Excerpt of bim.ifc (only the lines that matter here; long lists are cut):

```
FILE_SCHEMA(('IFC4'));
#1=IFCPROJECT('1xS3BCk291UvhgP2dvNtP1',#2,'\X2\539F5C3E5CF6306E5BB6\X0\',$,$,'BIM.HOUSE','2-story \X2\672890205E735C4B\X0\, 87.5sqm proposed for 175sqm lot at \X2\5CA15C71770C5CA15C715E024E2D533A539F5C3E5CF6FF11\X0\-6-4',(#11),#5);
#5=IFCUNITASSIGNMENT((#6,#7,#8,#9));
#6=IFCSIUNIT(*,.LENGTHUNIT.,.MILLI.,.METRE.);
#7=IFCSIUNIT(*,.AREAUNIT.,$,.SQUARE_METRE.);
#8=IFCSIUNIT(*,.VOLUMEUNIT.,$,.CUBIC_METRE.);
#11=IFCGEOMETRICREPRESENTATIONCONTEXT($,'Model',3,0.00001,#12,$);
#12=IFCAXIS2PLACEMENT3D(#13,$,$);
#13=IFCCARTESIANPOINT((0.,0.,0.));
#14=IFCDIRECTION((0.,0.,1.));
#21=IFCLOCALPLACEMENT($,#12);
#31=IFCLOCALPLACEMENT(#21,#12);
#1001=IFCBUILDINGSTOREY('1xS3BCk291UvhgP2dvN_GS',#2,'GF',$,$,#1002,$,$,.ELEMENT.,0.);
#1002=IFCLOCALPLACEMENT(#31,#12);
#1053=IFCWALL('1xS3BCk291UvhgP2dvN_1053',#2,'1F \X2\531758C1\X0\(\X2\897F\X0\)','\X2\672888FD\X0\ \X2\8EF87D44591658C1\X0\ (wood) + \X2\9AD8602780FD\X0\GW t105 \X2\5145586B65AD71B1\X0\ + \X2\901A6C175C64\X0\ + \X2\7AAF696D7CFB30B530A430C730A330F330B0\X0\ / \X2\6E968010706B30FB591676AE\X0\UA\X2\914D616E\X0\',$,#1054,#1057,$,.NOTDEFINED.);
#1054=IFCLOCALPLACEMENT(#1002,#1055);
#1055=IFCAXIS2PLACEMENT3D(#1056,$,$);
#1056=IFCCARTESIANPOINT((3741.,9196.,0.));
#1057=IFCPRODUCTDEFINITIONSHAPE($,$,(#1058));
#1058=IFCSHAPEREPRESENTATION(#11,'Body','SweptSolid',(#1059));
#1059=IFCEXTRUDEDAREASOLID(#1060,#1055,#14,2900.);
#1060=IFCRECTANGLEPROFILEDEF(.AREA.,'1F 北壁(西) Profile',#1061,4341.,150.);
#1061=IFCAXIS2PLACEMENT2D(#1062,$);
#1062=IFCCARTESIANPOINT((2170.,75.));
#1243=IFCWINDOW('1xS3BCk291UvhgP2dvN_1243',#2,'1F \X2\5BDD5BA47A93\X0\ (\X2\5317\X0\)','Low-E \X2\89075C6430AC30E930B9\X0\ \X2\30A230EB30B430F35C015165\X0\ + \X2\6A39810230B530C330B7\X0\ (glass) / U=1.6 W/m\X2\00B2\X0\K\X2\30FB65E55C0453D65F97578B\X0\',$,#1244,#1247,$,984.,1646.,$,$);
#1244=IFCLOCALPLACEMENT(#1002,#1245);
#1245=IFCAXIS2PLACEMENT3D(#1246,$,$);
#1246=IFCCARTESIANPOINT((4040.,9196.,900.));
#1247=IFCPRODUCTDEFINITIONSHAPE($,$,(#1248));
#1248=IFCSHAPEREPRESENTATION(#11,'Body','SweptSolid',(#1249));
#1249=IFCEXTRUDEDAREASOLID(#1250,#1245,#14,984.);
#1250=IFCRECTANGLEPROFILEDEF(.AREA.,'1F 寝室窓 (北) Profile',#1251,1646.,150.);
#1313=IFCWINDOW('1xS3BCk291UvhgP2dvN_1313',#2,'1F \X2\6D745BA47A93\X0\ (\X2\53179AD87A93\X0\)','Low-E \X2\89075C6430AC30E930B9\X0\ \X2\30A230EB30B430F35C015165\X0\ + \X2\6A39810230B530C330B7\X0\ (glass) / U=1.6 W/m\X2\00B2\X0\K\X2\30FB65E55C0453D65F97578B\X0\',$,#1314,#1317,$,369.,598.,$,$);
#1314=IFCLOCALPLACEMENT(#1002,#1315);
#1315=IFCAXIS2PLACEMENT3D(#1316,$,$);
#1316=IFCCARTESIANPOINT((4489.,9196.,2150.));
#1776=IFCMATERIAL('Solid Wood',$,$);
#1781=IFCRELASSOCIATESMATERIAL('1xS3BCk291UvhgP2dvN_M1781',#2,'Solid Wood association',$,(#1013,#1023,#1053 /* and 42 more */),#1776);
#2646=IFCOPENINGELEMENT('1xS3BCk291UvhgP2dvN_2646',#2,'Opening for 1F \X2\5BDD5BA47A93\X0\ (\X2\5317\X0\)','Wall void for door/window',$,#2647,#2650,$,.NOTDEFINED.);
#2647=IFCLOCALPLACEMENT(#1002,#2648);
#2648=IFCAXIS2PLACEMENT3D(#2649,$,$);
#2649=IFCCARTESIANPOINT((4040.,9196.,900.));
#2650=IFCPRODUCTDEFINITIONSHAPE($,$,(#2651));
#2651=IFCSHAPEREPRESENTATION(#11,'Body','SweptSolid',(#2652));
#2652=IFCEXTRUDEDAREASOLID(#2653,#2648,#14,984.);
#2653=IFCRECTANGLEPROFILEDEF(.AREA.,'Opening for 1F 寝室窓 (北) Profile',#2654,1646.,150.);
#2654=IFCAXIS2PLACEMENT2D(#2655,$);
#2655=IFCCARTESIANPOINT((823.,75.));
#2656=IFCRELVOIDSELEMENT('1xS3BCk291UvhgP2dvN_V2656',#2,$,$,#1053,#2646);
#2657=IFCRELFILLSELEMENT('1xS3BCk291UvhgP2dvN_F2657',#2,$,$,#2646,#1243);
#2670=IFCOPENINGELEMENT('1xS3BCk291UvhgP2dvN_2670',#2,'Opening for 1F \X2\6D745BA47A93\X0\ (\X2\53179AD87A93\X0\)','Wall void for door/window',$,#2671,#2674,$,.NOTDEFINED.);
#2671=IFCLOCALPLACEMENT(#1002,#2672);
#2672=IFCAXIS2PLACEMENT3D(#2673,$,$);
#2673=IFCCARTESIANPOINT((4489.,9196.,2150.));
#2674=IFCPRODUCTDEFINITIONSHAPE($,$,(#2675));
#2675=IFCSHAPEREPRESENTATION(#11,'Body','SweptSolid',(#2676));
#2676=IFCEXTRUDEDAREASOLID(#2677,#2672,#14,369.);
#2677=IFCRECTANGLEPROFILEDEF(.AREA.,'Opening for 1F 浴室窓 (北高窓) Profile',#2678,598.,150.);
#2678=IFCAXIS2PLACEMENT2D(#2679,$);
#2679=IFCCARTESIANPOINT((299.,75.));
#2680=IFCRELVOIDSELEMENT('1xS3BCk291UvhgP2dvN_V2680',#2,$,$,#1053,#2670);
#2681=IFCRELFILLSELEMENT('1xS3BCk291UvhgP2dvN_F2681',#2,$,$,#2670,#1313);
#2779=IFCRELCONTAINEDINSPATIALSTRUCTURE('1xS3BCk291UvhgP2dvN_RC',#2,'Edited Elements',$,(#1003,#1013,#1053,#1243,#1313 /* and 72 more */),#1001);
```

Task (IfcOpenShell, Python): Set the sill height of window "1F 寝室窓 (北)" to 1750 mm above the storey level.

```python
import numpy as np
import ifcopenshell
import ifcopenshell.api.geometry
import ifcopenshell.geom
import ifcopenshell.util.element
import ifcopenshell.util.placement
import ifcopenshell.util.shape
import ifcopenshell.util.unit

model = ifcopenshell.open("bim.ifc")
unit_scale = ifcopenshell.util.unit.calculate_unit_scale(model)

window = model.by_guid("1xS3BCk291UvhgP2dvN_1243")
opening = window.FillsVoids[0].RelatingOpeningElement
storey = ifcopenshell.util.element.get_container(window, ifc_class="IfcBuildingStorey")
level = ifcopenshell.util.placement.get_local_placement(storey.ObjectPlacement)[2, 3]

# The opening's origin need not be at the sill, so measure its lowest point.
shape = ifcopenshell.geom.create_shape(ifcopenshell.geom.settings(), opening)
bottom = ifcopenshell.util.shape.get_shape_bottom_elevation(shape, shape.geometry) / unit_scale
dz = level + 1750.0 - bottom

shift = np.array([0.0, 0.0, dz])
# The window is not placed relative to its opening, so move both.
for product in (opening, window):
    matrix = ifcopenshell.util.placement.get_local_placement(product.ObjectPlacement)
    matrix[:3, 3] += shift
    ifcopenshell.api.geometry.edit_object_placement(model, product=product, matrix=matrix, is_si=False)

print(f"moved by {dz * unit_scale:+.3f} m")

model.write("bim_v2.ifc")
```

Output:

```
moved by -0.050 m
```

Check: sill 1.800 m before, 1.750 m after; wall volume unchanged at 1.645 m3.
